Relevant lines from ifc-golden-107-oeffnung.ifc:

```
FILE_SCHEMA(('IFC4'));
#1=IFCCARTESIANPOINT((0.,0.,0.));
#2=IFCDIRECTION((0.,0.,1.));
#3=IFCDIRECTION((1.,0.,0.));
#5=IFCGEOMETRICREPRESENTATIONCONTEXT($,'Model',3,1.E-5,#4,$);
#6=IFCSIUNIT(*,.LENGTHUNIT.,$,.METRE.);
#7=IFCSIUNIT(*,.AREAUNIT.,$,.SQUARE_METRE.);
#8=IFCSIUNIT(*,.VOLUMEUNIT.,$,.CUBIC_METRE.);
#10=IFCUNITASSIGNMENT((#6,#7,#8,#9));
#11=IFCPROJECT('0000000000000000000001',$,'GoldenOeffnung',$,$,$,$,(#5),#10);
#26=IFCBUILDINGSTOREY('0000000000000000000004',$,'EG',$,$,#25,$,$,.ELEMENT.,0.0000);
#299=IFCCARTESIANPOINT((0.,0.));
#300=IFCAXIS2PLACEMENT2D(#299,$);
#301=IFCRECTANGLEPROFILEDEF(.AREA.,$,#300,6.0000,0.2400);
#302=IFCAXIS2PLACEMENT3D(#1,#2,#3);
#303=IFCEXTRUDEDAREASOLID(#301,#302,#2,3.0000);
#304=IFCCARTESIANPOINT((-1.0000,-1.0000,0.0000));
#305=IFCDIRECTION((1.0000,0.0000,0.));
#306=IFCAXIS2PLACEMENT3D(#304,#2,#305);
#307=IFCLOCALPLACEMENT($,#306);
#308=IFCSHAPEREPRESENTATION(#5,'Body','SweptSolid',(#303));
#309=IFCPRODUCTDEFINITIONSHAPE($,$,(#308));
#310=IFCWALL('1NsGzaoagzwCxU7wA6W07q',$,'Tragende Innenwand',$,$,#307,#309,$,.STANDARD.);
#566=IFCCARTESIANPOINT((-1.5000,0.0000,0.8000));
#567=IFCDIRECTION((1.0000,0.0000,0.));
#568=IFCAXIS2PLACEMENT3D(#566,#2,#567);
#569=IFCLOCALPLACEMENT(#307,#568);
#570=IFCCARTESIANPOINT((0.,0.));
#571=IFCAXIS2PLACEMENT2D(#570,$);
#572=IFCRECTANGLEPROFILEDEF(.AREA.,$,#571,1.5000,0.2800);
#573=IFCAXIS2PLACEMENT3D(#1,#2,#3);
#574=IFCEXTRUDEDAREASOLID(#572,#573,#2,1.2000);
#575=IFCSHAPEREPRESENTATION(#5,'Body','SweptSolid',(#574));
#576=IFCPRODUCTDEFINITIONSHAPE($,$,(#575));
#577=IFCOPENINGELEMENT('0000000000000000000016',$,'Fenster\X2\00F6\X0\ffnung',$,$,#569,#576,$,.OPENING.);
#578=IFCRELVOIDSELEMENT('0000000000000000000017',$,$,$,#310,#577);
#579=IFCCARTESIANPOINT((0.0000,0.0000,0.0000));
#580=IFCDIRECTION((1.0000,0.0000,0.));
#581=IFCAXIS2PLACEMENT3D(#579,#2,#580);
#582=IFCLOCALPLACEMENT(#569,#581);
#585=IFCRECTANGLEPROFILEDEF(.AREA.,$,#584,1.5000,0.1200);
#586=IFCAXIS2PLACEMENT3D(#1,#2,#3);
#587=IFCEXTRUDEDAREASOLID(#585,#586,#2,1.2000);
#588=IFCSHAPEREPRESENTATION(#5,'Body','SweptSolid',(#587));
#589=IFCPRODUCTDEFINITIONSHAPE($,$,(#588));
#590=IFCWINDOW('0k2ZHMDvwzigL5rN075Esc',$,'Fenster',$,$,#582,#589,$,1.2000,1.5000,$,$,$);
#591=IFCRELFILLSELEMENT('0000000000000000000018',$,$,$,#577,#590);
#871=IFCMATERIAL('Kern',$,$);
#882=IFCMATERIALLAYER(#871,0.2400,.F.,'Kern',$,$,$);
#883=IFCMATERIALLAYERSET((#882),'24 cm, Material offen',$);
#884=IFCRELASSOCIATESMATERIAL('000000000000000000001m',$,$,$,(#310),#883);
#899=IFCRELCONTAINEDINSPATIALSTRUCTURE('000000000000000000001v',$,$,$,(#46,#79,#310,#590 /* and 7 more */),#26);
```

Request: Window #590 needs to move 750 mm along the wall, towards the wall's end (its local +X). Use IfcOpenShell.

```python
import ifcopenshell
import ifcopenshell.api.geometry
import ifcopenshell.util.placement
import ifcopenshell.util.unit

model = ifcopenshell.open("ifc-golden-107-oeffnung.ifc")
unit_scale = ifcopenshell.util.unit.calculate_unit_scale(model)

window = model.by_id(590)
opening = window.FillsVoids[0].RelatingOpeningElement
wall = opening.VoidsElements[0].RelatingBuildingElement

wall_matrix = ifcopenshell.util.placement.get_local_placement(wall.ObjectPlacement)
shift = wall_matrix[:3, 0] * 0.75 / unit_scale
before = ifcopenshell.util.placement.get_local_placement(window.ObjectPlacement)[:3, 3].copy()

# The window is placed relative to its opening, so it follows when the opening moves.
matrix = ifcopenshell.util.placement.get_local_placement(opening.ObjectPlacement)
matrix[:3, 3] += shift
ifcopenshell.api.geometry.edit_object_placement(
    model, product=opening, matrix=matrix, is_si=False, should_transform_children=True
)

after = ifcopenshell.util.placement.get_local_placement(window.ObjectPlacement)[:3, 3]
print("window moved by", (after - before).round(3) + 0.0)

model.write("ifc-golden-107-oeffnung_updated.ifc")
```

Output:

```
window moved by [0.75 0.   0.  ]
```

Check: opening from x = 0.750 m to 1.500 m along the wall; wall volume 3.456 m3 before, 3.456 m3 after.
